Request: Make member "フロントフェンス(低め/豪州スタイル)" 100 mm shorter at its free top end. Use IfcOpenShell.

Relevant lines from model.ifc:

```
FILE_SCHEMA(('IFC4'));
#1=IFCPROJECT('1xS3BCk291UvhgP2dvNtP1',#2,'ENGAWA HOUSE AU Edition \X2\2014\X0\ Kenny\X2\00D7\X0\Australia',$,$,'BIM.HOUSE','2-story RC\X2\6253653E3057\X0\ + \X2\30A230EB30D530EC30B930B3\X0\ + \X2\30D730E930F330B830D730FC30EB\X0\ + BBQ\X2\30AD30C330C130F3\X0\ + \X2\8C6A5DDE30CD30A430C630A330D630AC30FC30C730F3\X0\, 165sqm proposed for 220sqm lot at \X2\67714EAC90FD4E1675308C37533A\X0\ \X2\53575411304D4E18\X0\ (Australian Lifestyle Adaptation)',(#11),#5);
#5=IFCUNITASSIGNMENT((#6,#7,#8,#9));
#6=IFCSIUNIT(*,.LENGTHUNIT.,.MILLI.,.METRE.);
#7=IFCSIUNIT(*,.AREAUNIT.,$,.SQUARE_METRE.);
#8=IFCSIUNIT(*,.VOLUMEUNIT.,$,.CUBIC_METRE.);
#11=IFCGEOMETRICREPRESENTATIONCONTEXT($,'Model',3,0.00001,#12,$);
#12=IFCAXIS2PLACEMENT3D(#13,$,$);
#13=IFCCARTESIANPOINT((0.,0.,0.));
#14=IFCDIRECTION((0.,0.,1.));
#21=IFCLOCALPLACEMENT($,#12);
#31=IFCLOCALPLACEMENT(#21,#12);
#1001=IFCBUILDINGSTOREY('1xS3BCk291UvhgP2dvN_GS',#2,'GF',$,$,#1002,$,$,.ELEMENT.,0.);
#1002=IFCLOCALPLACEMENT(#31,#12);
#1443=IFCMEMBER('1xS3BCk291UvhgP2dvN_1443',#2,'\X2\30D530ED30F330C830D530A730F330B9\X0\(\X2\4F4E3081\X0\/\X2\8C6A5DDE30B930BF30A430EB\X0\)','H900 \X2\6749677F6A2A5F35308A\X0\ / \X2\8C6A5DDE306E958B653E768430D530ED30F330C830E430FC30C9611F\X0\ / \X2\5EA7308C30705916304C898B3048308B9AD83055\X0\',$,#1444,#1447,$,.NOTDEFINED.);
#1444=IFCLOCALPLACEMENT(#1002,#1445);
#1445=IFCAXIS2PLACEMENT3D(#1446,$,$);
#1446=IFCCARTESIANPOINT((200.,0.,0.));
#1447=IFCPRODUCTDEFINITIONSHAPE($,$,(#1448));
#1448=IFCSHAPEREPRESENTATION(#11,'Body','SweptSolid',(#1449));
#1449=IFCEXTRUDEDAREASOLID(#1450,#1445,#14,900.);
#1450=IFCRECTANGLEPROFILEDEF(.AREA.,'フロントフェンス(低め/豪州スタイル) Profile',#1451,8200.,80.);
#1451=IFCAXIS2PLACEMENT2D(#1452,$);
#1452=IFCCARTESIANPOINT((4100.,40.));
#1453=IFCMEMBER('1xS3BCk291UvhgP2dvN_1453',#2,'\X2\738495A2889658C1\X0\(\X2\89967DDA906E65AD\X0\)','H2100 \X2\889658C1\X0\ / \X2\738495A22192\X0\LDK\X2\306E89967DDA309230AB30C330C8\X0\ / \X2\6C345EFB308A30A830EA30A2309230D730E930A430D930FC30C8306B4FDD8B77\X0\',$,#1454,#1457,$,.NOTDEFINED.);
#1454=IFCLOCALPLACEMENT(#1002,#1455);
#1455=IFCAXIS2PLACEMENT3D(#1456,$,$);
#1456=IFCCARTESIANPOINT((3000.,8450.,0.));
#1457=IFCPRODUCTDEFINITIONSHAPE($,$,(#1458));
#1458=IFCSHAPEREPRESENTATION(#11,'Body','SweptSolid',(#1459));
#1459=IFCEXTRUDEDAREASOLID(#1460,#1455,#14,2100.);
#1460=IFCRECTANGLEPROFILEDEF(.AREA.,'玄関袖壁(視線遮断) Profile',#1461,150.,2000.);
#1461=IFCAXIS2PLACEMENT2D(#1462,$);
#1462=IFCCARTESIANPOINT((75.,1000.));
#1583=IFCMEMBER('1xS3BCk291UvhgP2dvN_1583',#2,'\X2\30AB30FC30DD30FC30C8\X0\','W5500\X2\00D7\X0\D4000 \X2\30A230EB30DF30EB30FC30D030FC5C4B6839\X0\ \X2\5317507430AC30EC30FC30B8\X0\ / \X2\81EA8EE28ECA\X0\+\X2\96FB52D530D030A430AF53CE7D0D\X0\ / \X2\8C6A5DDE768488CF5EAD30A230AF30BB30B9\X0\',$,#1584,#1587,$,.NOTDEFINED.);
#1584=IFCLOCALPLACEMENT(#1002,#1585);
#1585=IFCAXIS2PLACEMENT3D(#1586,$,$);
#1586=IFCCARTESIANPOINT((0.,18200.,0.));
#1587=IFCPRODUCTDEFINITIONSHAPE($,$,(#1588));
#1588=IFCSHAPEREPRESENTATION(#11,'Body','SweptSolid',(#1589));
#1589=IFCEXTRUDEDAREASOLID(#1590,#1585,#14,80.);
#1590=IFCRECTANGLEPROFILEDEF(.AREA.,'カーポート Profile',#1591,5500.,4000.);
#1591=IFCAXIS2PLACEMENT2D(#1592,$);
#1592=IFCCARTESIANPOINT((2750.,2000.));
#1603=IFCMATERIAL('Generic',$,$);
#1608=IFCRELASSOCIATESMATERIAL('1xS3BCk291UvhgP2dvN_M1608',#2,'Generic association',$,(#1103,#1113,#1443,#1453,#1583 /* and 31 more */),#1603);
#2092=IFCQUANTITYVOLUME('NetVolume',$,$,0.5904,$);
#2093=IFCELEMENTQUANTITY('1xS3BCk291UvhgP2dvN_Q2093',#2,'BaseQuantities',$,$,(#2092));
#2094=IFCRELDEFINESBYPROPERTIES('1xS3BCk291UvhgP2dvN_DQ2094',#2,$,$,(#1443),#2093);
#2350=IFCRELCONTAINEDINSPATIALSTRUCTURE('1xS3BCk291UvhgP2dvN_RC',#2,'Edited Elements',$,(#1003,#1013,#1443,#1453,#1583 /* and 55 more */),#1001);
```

```python
import ifcopenshell
import ifcopenshell.api.pset
import ifcopenshell.util.element
import ifcopenshell.util.unit

model = ifcopenshell.open("model.ifc")
unit_scale = ifcopenshell.util.unit.calculate_unit_scale(model)

member = model.by_guid("1xS3BCk291UvhgP2dvN_1443")
change = -0.1 / unit_scale

# The extrusion runs towards the end named, so only its depth changes.
body = next(r for r in member.Representation.Representations if r.RepresentationIdentifier == "Body")
solid = body.Items[0]
old_length = solid.Depth
solid.Depth += change

# Update the stored length and volume.
qto = model.by_id(ifcopenshell.util.element.get_pset(member, "BaseQuantities", should_inherit=False)["id"])
ifcopenshell.api.pset.edit_qto(model, qto=qto, properties={
    "NetVolume": ifcopenshell.util.element.get_pset(member, "BaseQuantities", "NetVolume") * solid.Depth / old_length,
})

print(f"length {old_length:g} -> {solid.Depth:g}")

model.write("model_v2.ifc")
```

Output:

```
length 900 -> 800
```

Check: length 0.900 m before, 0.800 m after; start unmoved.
